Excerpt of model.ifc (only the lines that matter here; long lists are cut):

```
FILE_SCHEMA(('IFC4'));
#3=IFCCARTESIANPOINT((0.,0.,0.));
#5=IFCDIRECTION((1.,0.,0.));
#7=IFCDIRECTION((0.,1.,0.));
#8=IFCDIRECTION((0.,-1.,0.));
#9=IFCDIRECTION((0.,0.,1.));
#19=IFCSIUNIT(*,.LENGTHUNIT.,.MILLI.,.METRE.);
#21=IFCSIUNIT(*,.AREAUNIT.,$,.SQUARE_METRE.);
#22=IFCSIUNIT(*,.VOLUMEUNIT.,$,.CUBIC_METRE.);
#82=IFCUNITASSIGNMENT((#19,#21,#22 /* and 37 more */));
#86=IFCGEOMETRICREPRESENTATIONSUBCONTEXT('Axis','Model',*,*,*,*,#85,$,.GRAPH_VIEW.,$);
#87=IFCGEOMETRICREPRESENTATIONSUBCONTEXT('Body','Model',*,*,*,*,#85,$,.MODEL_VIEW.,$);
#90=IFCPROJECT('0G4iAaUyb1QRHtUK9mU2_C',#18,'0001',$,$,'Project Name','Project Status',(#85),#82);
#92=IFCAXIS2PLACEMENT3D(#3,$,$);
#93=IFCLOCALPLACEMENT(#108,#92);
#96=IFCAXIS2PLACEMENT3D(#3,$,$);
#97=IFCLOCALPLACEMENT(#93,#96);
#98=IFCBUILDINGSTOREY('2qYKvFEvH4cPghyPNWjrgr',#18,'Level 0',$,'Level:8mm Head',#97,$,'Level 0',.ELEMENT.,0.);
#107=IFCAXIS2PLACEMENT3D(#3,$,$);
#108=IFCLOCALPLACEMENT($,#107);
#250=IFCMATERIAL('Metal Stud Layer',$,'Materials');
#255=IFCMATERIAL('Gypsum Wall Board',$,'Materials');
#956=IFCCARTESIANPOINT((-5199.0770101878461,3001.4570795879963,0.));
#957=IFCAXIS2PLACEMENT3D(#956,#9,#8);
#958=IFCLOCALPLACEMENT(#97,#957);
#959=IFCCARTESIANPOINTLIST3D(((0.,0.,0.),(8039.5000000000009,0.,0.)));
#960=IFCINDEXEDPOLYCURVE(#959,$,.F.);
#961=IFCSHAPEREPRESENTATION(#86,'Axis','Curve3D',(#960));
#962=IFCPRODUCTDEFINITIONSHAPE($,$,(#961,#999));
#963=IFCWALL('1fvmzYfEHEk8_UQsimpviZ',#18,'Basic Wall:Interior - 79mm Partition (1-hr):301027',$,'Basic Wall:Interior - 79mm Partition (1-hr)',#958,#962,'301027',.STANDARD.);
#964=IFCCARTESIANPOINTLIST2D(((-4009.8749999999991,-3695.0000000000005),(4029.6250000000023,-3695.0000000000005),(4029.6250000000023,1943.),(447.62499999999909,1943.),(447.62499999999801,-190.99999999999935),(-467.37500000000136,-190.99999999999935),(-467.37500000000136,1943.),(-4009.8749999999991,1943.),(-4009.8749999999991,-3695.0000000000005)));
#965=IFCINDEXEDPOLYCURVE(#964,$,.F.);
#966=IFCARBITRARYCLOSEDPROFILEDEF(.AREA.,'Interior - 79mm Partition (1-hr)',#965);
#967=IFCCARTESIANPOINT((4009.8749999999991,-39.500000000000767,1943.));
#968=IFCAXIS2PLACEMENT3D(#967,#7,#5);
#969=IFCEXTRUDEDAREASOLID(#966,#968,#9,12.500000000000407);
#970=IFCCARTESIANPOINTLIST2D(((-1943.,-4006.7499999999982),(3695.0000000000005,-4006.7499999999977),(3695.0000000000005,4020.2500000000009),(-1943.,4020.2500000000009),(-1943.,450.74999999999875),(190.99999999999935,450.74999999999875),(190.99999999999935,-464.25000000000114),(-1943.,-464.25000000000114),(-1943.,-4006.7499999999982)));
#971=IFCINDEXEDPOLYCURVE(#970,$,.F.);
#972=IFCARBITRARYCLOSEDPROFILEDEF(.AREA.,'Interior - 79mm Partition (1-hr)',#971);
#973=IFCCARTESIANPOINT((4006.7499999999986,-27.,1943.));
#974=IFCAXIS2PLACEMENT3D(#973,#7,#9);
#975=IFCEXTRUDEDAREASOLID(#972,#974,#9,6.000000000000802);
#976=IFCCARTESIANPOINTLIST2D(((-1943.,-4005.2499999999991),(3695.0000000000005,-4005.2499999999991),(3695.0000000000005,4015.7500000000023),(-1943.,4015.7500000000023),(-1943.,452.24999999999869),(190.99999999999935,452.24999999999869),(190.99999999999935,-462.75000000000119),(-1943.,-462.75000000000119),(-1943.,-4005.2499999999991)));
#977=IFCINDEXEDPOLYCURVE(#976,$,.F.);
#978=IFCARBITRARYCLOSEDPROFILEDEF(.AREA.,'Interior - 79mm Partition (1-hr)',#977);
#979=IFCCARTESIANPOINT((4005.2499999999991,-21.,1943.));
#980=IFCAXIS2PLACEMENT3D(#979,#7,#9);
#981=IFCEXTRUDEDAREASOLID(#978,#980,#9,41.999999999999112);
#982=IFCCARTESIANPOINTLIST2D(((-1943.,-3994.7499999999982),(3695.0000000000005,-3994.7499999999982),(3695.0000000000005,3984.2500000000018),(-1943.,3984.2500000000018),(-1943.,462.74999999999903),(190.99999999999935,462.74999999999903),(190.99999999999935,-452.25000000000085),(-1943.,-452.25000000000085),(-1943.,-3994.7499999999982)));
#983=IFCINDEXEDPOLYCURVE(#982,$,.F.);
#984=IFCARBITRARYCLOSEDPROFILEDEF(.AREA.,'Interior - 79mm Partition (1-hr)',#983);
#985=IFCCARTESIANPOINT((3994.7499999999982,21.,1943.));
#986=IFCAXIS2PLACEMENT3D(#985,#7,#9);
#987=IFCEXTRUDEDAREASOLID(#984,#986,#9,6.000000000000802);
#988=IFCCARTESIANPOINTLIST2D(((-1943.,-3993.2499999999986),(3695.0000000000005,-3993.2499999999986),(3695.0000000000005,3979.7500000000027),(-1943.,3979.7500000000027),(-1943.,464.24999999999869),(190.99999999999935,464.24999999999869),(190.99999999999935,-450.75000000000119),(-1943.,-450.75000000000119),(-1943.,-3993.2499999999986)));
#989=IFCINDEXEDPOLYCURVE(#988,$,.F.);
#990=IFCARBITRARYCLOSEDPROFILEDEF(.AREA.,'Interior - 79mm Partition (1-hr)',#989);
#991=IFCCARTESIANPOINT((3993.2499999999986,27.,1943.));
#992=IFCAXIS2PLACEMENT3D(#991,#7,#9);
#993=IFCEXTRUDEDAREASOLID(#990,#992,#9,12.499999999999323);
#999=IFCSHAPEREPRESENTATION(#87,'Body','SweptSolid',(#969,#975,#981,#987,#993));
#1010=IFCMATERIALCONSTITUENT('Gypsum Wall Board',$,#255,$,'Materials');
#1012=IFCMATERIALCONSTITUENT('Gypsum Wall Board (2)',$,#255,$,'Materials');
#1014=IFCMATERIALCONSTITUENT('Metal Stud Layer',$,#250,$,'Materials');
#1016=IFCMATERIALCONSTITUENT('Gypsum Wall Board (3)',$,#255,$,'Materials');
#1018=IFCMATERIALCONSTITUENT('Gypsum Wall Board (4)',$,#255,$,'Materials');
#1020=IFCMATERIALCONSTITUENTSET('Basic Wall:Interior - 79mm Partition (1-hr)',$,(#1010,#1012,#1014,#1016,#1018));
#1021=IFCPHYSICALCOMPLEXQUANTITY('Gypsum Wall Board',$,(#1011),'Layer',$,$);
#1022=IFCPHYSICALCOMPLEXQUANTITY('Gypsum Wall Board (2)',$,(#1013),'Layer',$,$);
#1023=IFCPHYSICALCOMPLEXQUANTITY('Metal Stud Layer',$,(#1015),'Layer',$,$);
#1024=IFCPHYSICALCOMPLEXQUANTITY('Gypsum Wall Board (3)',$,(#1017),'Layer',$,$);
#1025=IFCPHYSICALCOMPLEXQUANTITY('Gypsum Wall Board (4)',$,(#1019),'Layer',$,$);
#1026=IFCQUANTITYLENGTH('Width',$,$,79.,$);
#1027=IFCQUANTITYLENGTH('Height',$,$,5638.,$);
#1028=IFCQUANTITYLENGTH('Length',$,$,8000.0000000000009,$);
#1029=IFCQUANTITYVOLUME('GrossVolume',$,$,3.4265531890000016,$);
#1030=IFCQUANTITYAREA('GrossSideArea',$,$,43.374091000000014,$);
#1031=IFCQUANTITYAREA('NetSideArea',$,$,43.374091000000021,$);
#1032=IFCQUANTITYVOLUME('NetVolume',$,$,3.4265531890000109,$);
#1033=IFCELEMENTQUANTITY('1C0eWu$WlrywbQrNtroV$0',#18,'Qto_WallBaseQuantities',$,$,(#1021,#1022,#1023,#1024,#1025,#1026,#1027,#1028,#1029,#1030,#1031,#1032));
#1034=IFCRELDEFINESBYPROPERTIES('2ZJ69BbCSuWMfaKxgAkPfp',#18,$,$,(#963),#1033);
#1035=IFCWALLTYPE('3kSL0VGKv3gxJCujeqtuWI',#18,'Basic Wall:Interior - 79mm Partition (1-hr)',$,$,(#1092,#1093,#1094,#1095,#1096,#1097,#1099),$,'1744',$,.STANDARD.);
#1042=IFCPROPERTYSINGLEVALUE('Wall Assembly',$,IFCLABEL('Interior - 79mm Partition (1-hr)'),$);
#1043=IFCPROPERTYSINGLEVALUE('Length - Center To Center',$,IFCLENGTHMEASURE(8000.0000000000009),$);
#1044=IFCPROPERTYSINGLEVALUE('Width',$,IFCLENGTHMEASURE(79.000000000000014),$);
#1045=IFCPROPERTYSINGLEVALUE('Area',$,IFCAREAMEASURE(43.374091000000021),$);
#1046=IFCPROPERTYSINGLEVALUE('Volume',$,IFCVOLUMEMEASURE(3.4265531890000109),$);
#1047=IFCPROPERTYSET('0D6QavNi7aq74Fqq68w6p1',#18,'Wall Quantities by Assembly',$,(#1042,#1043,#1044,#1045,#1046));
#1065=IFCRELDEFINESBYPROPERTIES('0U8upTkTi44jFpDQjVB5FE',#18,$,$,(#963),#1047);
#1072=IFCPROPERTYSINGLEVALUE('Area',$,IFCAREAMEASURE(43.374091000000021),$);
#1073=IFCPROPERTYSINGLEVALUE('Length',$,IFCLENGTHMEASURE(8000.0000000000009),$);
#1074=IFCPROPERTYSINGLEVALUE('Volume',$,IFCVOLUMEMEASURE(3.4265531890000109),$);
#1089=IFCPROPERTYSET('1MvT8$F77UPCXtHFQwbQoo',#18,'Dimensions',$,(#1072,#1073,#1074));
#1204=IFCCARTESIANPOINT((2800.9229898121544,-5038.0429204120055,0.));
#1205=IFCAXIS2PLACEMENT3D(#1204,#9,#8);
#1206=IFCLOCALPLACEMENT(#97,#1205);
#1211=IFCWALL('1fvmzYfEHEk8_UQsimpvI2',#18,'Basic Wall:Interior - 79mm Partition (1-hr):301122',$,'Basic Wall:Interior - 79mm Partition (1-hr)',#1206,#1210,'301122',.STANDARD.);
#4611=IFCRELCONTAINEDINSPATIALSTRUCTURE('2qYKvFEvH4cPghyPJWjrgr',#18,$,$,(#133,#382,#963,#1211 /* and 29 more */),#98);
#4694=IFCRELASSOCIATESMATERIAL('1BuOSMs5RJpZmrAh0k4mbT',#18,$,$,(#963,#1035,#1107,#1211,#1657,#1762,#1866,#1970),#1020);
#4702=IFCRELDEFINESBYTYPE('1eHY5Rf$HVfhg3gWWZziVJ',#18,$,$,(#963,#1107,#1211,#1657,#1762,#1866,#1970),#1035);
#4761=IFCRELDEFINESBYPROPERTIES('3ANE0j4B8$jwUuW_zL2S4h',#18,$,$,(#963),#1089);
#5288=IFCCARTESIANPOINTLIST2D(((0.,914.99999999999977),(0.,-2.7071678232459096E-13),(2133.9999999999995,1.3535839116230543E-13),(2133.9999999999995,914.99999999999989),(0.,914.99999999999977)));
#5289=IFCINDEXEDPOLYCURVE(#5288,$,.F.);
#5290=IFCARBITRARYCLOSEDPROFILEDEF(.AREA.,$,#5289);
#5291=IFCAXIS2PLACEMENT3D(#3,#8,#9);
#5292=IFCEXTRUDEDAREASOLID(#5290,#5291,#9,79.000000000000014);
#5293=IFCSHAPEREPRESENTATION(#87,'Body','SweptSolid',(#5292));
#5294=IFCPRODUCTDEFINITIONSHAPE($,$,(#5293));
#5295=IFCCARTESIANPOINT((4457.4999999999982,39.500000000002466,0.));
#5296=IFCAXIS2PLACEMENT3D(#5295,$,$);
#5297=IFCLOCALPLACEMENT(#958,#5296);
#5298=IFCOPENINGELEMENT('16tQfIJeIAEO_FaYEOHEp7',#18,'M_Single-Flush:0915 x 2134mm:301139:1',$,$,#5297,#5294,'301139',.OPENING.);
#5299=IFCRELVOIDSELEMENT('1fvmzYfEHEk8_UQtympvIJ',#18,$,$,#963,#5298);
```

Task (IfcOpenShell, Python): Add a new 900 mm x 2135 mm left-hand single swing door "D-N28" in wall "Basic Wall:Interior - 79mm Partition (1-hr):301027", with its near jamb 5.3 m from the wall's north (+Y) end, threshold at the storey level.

```python
import numpy as np
import ifcopenshell
import ifcopenshell.api.feature
import ifcopenshell.api.geometry
import ifcopenshell.api.pset
import ifcopenshell.api.root
import ifcopenshell.api.spatial
import ifcopenshell.geom
import ifcopenshell.util.element
import ifcopenshell.util.placement
import ifcopenshell.util.representation
import ifcopenshell.util.shape
import ifcopenshell.util.unit

model = ifcopenshell.open("model.ifc")
unit_scale = ifcopenshell.util.unit.calculate_unit_scale(model)
area_scale = ifcopenshell.util.unit.calculate_unit_scale(model, "AREAUNIT")
volume_scale = ifcopenshell.util.unit.calculate_unit_scale(model, "VOLUMEUNIT")
settings = ifcopenshell.geom.settings()


def volume(element):
    """Net volume in cubic metres, openings subtracted."""
    shape = ifcopenshell.geom.create_shape(settings, element)
    return ifcopenshell.util.shape.get_volume(shape.geometry)


wall = model.by_id(963)
storey = ifcopenshell.util.element.get_container(wall, ifc_class="IfcBuildingStorey")
context = ifcopenshell.util.representation.get_context(model, "Model", "Body", "MODEL_VIEW")
before = volume(wall)

width, height, from_end, sill = 0.9, 2.135, 5.3, 0.0  # metres

# The wall runs along its own X axis, and the end named is its -X end.
wall_shape = ifcopenshell.geom.create_shape(settings, wall)
x, y, z = ifcopenshell.util.shape.get_vertices(wall_shape.geometry).T
start = x.min() + from_end
face, thickness = float(y.min()), float(y.max() - y.min())
wall_matrix = ifcopenshell.util.placement.get_local_placement(wall.ObjectPlacement)
level = ifcopenshell.util.placement.get_local_placement(storey.ObjectPlacement)[2, 3]


def in_wall(x, y):
    """Placement at x, y metres in the wall's axes, at sill height."""
    matrix = wall_matrix.copy()
    matrix[:, 3] = wall_matrix @ np.array([x / unit_scale, y / unit_scale, 0.0, 1.0])
    matrix[2, 3] = level + sill / unit_scale
    return matrix


# Opening: a box that overshoots both wall faces by 50 mm.
opening = ifcopenshell.api.root.create_entity(model, ifc_class="IfcOpeningElement", predefined_type="OPENING")
box = ifcopenshell.api.geometry.add_wall_representation(
    model, context=context, length=width, height=height, thickness=thickness + 0.1
)
ifcopenshell.api.geometry.assign_representation(model, product=opening, representation=box)
ifcopenshell.api.geometry.edit_object_placement(model, product=opening, matrix=in_wall(start, face - 0.05), is_si=False)
ifcopenshell.api.feature.add_feature(model, feature=opening, element=wall)

door = ifcopenshell.api.root.create_entity(model, ifc_class="IfcDoor", name="D-N28", predefined_type="DOOR")
door.OverallWidth, door.OverallHeight = width / unit_scale, height / unit_scale
door.OperationType = "SINGLE_SWING_LEFT"
body = ifcopenshell.api.geometry.add_door_representation(
    model,
    context=context,
    overall_width=door.OverallWidth,
    overall_height=door.OverallHeight,
    operation_type="SINGLE_SWING_LEFT",
    lining_properties={"LiningDepth": thickness / unit_scale, "ThresholdDepth": thickness / unit_scale},
)
ifcopenshell.api.geometry.assign_representation(model, product=door, representation=body)
ifcopenshell.api.spatial.assign_container(model, products=[door], relating_structure=storey)
ifcopenshell.api.feature.add_filling(model, opening=opening, element=door)

# The lining spans the wall, so the door starts at the wall face.
ifcopenshell.api.geometry.edit_object_placement(model, product=door, matrix=in_wall(start, face), is_si=False)

after = volume(wall)

# Update the wall's stored quantities.
qto = model.by_id(ifcopenshell.util.element.get_pset(wall, "Qto_WallBaseQuantities", should_inherit=False)["id"])
ifcopenshell.api.pset.edit_qto(model, qto=qto, properties={
    "NetSideArea": after / thickness / area_scale,
    "NetVolume": after / volume_scale,
})
pset = model.by_id(ifcopenshell.util.element.get_pset(wall, "Wall Quantities by Assembly", should_inherit=False)["id"])
ifcopenshell.api.pset.edit_pset(model, pset=pset, properties={
    "Area": model.create_entity("IfcAreaMeasure", after / thickness / area_scale),
    "Volume": model.create_entity("IfcVolumeMeasure", after / volume_scale),
})
pset = model.by_id(ifcopenshell.util.element.get_pset(wall, "Dimensions", should_inherit=False)["id"])
ifcopenshell.api.pset.edit_pset(model, pset=pset, properties={
    "Area": model.create_entity("IfcAreaMeasure", after / thickness / area_scale),
    "Volume": model.create_entity("IfcVolumeMeasure", after / volume_scale),
})

print(f"wall volume {before:.3f} -> {after:.3f} m3")

model.write("model_updated.ifc")
```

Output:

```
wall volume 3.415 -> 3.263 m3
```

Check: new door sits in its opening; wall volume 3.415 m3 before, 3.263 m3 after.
